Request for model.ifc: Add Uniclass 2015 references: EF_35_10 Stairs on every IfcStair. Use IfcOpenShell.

First a look at what the model holds.

```python
import ifcopenshell

model = ifcopenshell.open("model.ifc")
print(model.schema)
print("classifications:", [c.Name for c in model.by_type("IfcClassification")])
for ifc_class in ("IfcDoor", "IfcRoof", "IfcStair", "IfcWall", "IfcWindow"):
    print(ifc_class, len(model.by_type(ifc_class)))
```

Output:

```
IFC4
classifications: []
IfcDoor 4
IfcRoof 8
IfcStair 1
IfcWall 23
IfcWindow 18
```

```python
import ifcopenshell
import ifcopenshell.api.classification

model = ifcopenshell.open("model.ifc")

system = ifcopenshell.api.classification.add_classification(model, classification="Uniclass 2015")

codes = {
    "IfcStair": ("EF_35_10", "Stairs"),
}
for ifc_class, (code, name) in codes.items():
    products = model.by_type(ifc_class)
    ifcopenshell.api.classification.add_reference(
        model, products=products, classification=system, identification=code, name=name
    )
    print(code, len(products))

model.write("model_edited.ifc")
```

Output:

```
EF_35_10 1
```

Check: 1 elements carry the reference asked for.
